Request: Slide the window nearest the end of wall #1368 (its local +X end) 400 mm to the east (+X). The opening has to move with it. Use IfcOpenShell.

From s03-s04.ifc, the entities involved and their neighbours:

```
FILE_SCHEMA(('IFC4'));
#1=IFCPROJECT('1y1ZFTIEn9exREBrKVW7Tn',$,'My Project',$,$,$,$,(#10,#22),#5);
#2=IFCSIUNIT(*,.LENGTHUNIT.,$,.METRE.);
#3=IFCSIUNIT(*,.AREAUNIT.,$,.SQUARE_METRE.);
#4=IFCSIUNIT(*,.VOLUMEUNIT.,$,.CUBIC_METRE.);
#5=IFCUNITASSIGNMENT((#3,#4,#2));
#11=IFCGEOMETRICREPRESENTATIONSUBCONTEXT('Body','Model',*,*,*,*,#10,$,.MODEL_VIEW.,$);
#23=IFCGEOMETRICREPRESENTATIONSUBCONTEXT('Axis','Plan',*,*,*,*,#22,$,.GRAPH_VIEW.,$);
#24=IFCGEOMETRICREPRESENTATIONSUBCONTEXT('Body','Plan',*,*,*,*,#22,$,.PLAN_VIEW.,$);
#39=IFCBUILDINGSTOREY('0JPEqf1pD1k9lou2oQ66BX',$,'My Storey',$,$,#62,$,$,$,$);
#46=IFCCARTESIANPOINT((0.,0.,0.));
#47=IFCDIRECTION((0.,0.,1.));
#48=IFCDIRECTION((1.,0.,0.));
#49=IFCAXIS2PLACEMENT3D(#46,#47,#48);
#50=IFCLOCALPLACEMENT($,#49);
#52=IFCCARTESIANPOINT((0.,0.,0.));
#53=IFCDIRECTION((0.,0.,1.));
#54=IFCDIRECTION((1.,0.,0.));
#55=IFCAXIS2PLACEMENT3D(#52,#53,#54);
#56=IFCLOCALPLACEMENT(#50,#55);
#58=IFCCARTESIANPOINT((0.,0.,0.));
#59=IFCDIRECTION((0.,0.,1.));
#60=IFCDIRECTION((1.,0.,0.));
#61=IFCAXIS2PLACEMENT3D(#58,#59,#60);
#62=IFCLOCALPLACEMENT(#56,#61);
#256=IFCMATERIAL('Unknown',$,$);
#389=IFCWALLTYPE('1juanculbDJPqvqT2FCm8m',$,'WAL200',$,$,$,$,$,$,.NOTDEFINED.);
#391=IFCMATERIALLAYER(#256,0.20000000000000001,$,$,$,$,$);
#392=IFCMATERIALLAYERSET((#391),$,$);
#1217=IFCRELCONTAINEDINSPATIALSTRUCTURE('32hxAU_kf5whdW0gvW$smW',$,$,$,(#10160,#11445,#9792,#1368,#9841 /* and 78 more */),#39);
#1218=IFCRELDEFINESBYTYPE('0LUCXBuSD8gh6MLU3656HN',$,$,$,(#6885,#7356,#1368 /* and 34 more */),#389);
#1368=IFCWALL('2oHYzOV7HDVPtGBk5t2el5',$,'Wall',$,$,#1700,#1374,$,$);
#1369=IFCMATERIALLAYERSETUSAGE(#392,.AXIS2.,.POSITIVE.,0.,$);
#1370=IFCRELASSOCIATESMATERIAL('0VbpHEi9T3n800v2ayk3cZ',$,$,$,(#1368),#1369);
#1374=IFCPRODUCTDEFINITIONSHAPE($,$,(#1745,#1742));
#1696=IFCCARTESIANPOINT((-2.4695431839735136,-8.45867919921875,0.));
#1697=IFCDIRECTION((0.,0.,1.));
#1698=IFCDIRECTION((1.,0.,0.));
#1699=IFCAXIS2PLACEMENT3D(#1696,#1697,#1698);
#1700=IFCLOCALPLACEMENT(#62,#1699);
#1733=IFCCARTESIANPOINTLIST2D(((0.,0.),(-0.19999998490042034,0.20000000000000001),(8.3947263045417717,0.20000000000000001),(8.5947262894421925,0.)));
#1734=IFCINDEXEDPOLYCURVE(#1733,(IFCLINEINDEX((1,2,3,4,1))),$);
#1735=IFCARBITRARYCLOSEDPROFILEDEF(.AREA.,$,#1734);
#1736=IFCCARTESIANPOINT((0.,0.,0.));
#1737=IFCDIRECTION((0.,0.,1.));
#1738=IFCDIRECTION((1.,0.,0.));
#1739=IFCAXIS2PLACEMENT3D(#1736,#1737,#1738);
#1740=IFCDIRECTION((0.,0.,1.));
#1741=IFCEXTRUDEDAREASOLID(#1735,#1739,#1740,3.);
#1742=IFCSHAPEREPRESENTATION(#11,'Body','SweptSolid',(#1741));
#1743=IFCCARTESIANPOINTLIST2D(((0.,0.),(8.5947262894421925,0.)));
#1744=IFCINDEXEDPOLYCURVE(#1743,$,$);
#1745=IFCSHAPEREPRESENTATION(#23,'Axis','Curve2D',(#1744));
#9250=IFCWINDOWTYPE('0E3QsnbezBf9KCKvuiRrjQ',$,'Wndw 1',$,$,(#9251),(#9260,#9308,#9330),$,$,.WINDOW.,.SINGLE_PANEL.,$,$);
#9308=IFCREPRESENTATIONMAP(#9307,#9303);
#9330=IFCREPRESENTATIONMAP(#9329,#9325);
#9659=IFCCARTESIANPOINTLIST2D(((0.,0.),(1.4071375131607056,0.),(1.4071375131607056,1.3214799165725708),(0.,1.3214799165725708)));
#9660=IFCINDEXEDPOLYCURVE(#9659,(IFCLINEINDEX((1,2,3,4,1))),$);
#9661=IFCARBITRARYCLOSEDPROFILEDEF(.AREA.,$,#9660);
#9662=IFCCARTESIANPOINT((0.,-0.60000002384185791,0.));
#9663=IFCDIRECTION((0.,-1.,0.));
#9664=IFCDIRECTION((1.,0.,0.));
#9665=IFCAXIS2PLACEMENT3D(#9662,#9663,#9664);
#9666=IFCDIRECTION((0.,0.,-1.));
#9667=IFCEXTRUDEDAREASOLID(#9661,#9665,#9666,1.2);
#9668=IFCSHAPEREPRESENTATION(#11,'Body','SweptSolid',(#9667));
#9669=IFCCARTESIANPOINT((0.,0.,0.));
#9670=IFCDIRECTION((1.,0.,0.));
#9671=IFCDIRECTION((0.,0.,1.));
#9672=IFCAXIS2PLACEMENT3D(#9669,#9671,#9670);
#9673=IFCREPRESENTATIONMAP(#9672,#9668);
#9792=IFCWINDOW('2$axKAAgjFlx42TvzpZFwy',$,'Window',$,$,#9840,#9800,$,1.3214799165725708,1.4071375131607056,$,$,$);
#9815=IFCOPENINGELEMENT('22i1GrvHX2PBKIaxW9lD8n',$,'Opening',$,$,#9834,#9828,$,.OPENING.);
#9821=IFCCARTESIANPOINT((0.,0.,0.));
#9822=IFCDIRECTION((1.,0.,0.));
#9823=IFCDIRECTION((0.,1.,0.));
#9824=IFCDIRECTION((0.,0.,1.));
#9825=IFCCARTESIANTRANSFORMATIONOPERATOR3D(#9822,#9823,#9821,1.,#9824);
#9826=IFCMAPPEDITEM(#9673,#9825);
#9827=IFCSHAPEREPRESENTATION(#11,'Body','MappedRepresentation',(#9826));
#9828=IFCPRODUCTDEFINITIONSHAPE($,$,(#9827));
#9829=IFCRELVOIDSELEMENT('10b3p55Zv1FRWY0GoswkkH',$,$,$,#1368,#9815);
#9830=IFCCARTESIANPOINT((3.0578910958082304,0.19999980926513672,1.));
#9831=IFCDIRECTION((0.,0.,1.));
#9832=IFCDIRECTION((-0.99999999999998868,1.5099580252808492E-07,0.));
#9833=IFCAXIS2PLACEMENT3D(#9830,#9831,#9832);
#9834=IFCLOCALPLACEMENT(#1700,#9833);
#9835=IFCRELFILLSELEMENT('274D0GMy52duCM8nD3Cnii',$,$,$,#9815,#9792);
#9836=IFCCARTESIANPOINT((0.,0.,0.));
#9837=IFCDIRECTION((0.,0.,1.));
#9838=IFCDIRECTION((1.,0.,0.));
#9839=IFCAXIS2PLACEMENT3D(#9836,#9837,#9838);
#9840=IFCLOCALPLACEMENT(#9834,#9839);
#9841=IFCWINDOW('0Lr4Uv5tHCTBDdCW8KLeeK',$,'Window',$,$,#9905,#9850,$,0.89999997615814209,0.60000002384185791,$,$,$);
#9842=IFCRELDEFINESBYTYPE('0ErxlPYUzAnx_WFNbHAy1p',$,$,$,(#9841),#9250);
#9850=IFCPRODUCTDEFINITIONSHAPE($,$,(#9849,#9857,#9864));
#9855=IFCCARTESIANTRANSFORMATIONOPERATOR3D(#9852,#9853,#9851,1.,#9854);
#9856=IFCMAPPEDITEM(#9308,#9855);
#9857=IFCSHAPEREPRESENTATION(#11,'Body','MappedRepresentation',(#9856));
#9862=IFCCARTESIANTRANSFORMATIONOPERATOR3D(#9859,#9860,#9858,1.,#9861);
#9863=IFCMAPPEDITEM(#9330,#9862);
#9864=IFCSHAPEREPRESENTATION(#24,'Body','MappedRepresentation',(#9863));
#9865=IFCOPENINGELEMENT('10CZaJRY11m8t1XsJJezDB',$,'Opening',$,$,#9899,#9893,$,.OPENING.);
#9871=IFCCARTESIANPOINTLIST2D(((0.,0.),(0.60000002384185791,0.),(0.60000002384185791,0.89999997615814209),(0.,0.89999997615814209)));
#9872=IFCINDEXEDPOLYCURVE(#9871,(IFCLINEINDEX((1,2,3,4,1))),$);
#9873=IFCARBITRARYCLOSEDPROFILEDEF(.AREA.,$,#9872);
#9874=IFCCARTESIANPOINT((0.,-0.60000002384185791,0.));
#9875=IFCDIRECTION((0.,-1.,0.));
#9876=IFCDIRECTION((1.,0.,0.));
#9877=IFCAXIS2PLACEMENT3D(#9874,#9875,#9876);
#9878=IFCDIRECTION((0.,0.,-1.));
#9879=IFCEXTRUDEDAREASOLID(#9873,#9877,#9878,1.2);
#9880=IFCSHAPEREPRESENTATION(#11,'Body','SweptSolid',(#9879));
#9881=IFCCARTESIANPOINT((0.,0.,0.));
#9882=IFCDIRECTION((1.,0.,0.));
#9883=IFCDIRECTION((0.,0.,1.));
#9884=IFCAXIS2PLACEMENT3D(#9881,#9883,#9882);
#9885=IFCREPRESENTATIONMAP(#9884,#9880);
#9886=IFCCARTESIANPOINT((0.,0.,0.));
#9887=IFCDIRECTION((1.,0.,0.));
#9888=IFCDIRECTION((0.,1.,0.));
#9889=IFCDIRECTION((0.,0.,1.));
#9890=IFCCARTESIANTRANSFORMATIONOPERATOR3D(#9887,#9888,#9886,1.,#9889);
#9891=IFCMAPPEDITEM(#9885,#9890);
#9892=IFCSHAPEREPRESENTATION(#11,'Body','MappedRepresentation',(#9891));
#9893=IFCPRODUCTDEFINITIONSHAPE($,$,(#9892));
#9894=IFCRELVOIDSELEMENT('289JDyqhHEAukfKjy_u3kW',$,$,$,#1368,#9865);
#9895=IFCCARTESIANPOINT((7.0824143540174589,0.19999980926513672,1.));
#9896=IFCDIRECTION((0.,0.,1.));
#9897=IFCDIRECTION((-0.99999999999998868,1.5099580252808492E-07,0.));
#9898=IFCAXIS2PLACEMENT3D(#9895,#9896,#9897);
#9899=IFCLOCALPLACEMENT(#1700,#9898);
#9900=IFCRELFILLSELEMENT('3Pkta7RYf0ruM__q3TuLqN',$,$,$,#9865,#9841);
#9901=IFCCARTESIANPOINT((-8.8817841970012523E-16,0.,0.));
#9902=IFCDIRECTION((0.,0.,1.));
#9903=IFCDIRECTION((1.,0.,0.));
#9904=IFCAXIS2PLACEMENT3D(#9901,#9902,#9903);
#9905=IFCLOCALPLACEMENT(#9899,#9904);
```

```python
import ifcopenshell
import ifcopenshell.api.geometry
import ifcopenshell.util.placement
import ifcopenshell.util.unit

model = ifcopenshell.open("s03-s04.ifc")
unit_scale = ifcopenshell.util.unit.calculate_unit_scale(model)

window = model.by_id(9841)
opening = window.FillsVoids[0].RelatingOpeningElement
wall = opening.VoidsElements[0].RelatingBuildingElement

wall_matrix = ifcopenshell.util.placement.get_local_placement(wall.ObjectPlacement)
shift = wall_matrix[:3, 0] * 0.4 / unit_scale
before = ifcopenshell.util.placement.get_local_placement(window.ObjectPlacement)[:3, 3].copy()

# The window is placed relative to its opening, so it follows when the opening moves.
matrix = ifcopenshell.util.placement.get_local_placement(opening.ObjectPlacement)
matrix[:3, 3] += shift
ifcopenshell.api.geometry.edit_object_placement(
    model, product=opening, matrix=matrix, is_si=False, should_transform_children=True
)

after = ifcopenshell.util.placement.get_local_placement(window.ObjectPlacement)[:3, 3]
print("window moved by", (after - before).round(3) + 0.0)

model.write("s03-s04_v2.ifc")
```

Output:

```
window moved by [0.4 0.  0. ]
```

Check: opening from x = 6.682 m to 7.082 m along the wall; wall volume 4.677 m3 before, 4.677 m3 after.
